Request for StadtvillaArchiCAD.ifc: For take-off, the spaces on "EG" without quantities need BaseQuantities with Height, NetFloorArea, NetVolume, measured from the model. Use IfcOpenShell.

First a look at what the model holds.

```python
import ifcopenshell
import ifcopenshell.util.element
import ifcopenshell.util.unit

model = ifcopenshell.open("StadtvillaArchiCAD.ifc")
print(model.schema)
for unit_type in ("LENGTHUNIT", "AREAUNIT", "VOLUMEUNIT"):
    print(unit_type, ifcopenshell.util.unit.calculate_unit_scale(model, unit_type))
storey = next(s for s in model.by_type("IfcBuildingStorey") if s.Name == "EG")
spaces = [e for e in ifcopenshell.util.element.get_decomposition(storey) if e.is_a("IfcSpace")]
for e in sorted(spaces, key=lambda e: e.id()):
    print(e.id(), e.is_a(), e.Name, list(ifcopenshell.util.element.get_psets(e, qtos_only=True)), sep=" | ")
```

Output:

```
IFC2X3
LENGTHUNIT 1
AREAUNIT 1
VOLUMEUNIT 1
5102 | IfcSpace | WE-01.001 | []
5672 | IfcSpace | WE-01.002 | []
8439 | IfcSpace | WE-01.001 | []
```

```python
import ifcopenshell
import ifcopenshell.api.pset
import ifcopenshell.geom
import ifcopenshell.util.element
import ifcopenshell.util.shape
import ifcopenshell.util.unit

model = ifcopenshell.open("StadtvillaArchiCAD.ifc")
unit_scale = ifcopenshell.util.unit.calculate_unit_scale(model)
area_scale = ifcopenshell.util.unit.calculate_unit_scale(model, "AREAUNIT")
volume_scale = ifcopenshell.util.unit.calculate_unit_scale(model, "VOLUMEUNIT")
settings = ifcopenshell.geom.settings()

storey = next(s for s in model.by_type("IfcBuildingStorey") if s.Name == "EG")
spaces = [e for e in ifcopenshell.util.element.get_decomposition(storey) if e.is_a("IfcSpace")]

for e in sorted(spaces, key=lambda e: e.id()):
    if ifcopenshell.util.element.get_psets(e, qtos_only=True, should_inherit=False):
        continue
    # Geometry comes back in metres, in the element's own axes.
    shape = ifcopenshell.geom.create_shape(settings, e)
    values = {
        "Height": ifcopenshell.util.shape.get_z(shape.geometry) / unit_scale,
        "NetFloorArea": ifcopenshell.util.shape.get_footprint_area(shape.geometry) / area_scale,
        "NetVolume": ifcopenshell.util.shape.get_volume(shape.geometry) / volume_scale,
    }
    qto = ifcopenshell.api.pset.add_qto(model, product=e, name="BaseQuantities")
    ifcopenshell.api.pset.edit_qto(model, qto=qto, properties=values)
    print(e.id(), {k: round(v, 3) for k, v in values.items()})

model.write("StadtvillaArchiCAD_rev.ifc")
```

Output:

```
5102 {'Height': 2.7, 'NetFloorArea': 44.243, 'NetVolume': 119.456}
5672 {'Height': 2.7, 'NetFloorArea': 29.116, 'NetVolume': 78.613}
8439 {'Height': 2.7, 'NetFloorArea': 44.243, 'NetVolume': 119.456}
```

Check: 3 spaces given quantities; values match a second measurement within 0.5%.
